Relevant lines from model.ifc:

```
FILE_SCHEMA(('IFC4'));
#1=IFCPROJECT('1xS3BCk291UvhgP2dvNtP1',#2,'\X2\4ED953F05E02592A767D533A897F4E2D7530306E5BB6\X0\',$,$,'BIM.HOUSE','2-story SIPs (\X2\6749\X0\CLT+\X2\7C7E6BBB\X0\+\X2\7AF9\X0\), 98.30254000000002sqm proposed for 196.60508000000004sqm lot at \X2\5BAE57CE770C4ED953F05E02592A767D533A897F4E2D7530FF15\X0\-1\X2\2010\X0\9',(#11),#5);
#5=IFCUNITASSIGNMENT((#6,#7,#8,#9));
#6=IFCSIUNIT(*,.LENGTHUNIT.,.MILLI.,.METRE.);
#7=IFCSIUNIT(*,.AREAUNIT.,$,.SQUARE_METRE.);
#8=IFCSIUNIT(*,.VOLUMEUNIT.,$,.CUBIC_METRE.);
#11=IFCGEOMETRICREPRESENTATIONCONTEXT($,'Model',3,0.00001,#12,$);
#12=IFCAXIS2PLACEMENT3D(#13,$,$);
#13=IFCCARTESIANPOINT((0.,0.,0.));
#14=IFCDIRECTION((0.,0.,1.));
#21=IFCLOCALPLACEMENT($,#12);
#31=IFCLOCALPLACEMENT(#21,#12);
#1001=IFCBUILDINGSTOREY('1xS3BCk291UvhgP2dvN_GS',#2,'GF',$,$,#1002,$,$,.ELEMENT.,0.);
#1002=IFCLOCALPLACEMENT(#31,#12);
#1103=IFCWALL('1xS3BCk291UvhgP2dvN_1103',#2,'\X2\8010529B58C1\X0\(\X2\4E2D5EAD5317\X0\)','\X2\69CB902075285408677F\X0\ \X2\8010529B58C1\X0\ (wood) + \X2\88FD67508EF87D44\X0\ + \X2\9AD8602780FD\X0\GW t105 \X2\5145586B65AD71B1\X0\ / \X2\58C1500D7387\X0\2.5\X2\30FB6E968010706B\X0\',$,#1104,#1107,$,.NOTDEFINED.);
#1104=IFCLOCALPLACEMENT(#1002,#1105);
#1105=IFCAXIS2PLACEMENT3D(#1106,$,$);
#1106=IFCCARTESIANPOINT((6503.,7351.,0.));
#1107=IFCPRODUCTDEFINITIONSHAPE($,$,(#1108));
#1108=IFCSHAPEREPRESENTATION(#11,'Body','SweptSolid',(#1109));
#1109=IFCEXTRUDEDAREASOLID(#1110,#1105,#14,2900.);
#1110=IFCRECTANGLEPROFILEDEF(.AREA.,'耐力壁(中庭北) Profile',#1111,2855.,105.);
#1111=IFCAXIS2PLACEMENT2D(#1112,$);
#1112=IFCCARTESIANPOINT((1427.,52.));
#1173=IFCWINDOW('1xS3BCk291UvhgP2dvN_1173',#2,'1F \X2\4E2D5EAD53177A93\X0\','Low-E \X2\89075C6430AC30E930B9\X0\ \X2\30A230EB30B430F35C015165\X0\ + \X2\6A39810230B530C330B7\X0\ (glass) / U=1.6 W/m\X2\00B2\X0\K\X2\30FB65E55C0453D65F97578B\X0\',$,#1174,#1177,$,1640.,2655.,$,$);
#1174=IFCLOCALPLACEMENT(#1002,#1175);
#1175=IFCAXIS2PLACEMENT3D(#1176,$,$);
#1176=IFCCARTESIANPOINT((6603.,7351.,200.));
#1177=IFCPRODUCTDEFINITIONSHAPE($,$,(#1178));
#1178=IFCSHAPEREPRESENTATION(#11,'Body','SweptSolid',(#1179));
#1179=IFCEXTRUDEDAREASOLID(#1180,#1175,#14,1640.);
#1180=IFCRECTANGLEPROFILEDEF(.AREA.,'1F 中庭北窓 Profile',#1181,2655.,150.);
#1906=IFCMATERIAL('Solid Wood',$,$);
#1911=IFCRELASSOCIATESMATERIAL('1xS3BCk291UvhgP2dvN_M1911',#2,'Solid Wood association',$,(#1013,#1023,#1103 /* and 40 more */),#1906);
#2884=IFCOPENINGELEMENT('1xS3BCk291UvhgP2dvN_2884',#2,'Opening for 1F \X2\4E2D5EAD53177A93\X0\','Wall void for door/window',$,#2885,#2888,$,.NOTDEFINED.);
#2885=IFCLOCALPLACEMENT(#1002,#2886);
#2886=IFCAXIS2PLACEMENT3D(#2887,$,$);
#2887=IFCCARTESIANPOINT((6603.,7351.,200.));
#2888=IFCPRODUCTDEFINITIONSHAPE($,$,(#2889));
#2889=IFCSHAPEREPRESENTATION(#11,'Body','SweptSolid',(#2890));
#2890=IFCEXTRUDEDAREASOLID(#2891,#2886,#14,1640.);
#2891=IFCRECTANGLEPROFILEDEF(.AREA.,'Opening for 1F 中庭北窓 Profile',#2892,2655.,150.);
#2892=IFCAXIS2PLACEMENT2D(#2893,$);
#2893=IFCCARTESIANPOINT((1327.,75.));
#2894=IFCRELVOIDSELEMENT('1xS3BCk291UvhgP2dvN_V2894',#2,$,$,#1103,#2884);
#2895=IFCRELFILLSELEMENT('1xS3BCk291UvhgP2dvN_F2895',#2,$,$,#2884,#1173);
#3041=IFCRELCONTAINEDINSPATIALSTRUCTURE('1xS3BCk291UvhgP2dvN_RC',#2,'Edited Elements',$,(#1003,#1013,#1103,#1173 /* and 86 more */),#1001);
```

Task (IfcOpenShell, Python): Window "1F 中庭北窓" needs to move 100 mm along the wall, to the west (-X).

```python
import ifcopenshell
import ifcopenshell.api.geometry
import ifcopenshell.util.placement
import ifcopenshell.util.unit

model = ifcopenshell.open("model.ifc")
unit_scale = ifcopenshell.util.unit.calculate_unit_scale(model)

window = model.by_guid("1xS3BCk291UvhgP2dvN_1173")
opening = window.FillsVoids[0].RelatingOpeningElement
wall = opening.VoidsElements[0].RelatingBuildingElement

wall_matrix = ifcopenshell.util.placement.get_local_placement(wall.ObjectPlacement)
shift = wall_matrix[:3, 0] * -0.1 / unit_scale
before = ifcopenshell.util.placement.get_local_placement(window.ObjectPlacement)[:3, 3].copy()

# The window is not placed relative to its opening, so move both.
for product in (opening, window):
    matrix = ifcopenshell.util.placement.get_local_placement(product.ObjectPlacement)
    matrix[:3, 3] += shift
    ifcopenshell.api.geometry.edit_object_placement(model, product=product, matrix=matrix, is_si=False)

after = ifcopenshell.util.placement.get_local_placement(window.ObjectPlacement)[:3, 3]
print("window moved by", (after - before).round(3) + 0.0)

model.write("model-out.ifc")
```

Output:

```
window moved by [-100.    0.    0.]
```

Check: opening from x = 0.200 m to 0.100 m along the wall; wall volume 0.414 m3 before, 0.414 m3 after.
